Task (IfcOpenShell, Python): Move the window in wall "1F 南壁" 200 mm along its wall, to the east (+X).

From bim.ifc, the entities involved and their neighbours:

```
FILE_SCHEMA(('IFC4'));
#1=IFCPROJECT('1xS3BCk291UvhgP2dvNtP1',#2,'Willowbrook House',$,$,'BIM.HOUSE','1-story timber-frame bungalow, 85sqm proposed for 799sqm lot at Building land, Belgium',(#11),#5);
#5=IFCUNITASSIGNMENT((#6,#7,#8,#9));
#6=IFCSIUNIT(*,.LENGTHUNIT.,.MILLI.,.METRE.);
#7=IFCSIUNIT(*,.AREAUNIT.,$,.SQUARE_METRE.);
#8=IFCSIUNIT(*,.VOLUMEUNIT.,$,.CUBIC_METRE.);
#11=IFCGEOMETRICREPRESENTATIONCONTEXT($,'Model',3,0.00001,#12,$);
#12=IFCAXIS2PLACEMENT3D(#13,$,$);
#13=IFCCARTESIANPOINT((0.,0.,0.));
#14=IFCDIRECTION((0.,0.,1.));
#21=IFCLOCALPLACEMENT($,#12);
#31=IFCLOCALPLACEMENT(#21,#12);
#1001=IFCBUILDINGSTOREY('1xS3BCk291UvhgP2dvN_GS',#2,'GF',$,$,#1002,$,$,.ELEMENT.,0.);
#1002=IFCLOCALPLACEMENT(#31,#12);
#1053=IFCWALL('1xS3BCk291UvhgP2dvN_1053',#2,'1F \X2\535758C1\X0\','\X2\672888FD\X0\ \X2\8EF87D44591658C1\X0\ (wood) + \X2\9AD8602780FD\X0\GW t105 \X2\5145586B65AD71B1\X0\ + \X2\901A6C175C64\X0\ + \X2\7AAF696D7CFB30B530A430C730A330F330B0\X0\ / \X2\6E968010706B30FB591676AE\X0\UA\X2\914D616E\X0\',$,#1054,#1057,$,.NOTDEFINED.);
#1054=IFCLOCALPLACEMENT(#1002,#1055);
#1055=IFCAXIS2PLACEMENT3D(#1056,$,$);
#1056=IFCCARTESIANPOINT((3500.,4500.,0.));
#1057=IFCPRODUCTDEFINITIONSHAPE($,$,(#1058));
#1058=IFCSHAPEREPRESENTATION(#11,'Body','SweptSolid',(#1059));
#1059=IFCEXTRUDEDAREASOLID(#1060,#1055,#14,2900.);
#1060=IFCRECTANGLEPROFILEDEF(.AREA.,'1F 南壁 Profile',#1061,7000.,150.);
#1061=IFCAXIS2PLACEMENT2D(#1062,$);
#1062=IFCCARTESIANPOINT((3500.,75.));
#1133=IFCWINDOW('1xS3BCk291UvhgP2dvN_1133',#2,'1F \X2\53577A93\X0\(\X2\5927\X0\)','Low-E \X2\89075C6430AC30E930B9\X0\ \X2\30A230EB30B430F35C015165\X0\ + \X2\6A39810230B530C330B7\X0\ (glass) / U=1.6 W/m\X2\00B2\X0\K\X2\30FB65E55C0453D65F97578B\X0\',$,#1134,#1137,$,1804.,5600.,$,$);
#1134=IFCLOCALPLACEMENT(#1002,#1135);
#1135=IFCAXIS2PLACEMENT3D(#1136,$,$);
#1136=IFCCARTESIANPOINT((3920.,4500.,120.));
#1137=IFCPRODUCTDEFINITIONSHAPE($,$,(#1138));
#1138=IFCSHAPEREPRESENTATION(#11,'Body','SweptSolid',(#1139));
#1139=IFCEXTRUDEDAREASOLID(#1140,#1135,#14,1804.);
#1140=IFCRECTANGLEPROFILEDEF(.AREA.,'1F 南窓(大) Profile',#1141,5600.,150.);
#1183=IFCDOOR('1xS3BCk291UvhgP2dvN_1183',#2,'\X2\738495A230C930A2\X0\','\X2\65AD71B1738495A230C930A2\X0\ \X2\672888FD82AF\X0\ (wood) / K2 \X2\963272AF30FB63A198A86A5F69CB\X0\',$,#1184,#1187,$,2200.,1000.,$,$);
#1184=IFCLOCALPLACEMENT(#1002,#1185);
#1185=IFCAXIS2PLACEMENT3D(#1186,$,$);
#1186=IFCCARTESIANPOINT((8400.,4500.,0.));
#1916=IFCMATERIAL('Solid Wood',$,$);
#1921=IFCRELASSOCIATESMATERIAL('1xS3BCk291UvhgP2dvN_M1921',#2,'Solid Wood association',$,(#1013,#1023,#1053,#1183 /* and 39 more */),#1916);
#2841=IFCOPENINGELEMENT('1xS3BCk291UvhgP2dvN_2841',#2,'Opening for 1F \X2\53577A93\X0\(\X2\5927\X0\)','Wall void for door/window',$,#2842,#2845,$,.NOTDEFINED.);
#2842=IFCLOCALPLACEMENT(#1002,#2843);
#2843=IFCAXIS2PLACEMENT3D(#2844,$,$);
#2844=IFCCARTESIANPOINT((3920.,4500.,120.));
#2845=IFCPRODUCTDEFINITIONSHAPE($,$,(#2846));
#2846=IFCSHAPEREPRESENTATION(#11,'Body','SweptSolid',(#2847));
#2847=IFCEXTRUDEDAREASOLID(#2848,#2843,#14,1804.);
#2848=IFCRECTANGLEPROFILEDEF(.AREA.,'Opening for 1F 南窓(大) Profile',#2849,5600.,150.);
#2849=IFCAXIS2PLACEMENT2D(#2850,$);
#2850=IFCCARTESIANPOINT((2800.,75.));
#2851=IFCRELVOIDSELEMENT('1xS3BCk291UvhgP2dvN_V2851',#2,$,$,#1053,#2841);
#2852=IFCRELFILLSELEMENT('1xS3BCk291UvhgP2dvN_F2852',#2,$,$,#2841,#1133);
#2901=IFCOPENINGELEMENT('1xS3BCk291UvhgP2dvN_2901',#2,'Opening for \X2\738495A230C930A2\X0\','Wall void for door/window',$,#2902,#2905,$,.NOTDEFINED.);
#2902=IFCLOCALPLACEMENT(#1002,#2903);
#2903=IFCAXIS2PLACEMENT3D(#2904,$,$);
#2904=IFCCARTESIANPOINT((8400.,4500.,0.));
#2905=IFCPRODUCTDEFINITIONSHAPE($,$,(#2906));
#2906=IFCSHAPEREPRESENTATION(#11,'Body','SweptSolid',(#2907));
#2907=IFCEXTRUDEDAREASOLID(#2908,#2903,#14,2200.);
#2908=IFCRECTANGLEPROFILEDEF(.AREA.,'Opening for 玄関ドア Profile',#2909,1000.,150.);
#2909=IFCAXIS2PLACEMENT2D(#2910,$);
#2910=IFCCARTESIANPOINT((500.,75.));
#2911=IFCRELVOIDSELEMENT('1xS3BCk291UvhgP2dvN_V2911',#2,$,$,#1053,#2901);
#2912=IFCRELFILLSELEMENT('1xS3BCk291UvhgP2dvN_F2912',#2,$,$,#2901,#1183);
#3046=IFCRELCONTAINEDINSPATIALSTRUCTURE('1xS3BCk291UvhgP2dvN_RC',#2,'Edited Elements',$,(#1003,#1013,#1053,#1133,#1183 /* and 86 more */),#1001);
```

```python
import ifcopenshell
import ifcopenshell.api.geometry
import ifcopenshell.util.placement
import ifcopenshell.util.unit

model = ifcopenshell.open("bim.ifc")
unit_scale = ifcopenshell.util.unit.calculate_unit_scale(model)

window = model.by_guid("1xS3BCk291UvhgP2dvN_1133")
opening = window.FillsVoids[0].RelatingOpeningElement
wall = opening.VoidsElements[0].RelatingBuildingElement

wall_matrix = ifcopenshell.util.placement.get_local_placement(wall.ObjectPlacement)
shift = wall_matrix[:3, 0] * 0.2 / unit_scale
before = ifcopenshell.util.placement.get_local_placement(window.ObjectPlacement)[:3, 3].copy()

# The window is not placed relative to its opening, so move both.
for product in (opening, window):
    matrix = ifcopenshell.util.placement.get_local_placement(product.ObjectPlacement)
    matrix[:3, 3] += shift
    ifcopenshell.api.geometry.edit_object_placement(model, product=product, matrix=matrix, is_si=False)

after = ifcopenshell.util.placement.get_local_placement(window.ObjectPlacement)[:3, 3]
print("window moved by", (after - before).round(3) + 0.0)

model.write("bim_edited.ifc")
```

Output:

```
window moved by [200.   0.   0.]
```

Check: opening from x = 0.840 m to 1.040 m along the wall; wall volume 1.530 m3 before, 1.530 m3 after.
